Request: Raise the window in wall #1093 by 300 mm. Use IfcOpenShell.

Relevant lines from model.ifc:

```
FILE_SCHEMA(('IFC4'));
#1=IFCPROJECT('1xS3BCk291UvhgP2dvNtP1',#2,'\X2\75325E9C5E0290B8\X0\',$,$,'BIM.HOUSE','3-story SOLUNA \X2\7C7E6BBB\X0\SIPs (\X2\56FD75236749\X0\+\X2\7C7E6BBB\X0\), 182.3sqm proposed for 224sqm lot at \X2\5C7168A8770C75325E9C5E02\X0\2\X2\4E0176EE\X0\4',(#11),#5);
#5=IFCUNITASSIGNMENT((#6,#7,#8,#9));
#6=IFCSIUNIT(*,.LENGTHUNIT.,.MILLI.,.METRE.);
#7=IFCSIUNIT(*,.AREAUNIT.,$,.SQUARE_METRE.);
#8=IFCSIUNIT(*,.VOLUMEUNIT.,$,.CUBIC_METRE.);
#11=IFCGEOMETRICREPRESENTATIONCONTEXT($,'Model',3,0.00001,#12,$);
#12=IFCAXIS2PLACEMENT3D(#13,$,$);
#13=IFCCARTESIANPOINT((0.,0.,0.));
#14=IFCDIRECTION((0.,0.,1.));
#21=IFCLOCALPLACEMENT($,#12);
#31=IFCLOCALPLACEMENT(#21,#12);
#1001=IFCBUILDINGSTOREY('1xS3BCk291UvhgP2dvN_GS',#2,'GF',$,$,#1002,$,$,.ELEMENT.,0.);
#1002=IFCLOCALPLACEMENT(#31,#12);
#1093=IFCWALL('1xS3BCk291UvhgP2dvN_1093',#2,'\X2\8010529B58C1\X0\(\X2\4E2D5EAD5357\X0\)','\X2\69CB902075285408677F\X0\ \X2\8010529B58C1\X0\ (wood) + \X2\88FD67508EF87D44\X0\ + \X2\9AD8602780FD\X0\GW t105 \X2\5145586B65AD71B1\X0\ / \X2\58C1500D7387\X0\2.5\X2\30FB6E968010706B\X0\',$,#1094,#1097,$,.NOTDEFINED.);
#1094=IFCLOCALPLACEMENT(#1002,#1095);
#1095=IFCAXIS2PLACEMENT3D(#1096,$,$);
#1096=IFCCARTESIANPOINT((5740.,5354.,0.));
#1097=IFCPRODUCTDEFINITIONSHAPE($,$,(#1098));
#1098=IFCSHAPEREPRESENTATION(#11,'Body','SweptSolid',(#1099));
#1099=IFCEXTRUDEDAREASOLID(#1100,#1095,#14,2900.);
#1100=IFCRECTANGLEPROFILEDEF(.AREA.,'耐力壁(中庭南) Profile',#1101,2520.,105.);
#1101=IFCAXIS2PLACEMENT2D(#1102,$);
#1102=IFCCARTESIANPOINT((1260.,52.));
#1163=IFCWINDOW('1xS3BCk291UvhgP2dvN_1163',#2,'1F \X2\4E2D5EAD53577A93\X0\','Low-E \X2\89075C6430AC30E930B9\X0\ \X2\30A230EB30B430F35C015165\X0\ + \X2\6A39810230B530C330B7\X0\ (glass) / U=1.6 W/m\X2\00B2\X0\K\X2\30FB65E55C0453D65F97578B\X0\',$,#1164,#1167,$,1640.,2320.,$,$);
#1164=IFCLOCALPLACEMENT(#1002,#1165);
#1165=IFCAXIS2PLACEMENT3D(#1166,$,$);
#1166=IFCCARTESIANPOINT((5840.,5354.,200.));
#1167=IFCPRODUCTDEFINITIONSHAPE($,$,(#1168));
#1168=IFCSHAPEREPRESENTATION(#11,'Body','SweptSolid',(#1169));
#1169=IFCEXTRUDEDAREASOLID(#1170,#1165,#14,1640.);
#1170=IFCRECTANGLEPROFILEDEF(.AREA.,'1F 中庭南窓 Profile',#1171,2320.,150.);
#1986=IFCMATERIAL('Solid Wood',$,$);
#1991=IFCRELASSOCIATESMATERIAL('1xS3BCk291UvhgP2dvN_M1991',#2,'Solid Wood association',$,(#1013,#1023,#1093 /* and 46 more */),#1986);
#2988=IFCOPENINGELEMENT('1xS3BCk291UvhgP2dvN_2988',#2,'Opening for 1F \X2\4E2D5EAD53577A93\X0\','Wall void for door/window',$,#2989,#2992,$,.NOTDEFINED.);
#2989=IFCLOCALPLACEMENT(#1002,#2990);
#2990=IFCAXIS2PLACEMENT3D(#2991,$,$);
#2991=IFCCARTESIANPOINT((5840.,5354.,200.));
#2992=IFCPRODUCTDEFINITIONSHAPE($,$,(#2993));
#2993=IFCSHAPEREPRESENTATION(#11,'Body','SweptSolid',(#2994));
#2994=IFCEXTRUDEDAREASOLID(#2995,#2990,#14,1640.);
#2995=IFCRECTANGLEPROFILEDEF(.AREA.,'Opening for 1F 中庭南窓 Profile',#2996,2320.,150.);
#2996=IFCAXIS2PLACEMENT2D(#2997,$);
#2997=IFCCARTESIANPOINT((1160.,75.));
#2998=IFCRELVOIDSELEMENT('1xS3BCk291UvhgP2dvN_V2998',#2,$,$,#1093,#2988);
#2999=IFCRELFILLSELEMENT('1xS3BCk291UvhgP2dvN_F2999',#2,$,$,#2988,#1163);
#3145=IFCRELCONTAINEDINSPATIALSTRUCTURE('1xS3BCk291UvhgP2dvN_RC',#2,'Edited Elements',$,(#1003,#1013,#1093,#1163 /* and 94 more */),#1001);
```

```python
import numpy as np
import ifcopenshell
import ifcopenshell.api.geometry
import ifcopenshell.util.placement
import ifcopenshell.util.unit

model = ifcopenshell.open("model.ifc")
unit_scale = ifcopenshell.util.unit.calculate_unit_scale(model)

window = model.by_guid("1xS3BCk291UvhgP2dvN_1163")
opening = window.FillsVoids[0].RelatingOpeningElement
dz = 0.3 / unit_scale

shift = np.array([0.0, 0.0, dz])
# The window is not placed relative to its opening, so move both.
for product in (opening, window):
    matrix = ifcopenshell.util.placement.get_local_placement(product.ObjectPlacement)
    matrix[:3, 3] += shift
    ifcopenshell.api.geometry.edit_object_placement(model, product=product, matrix=matrix, is_si=False)

print(f"moved by {dz * unit_scale:+.3f} m")

model.write("model_rev.ifc")
```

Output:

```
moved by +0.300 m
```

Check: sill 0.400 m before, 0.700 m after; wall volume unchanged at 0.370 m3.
